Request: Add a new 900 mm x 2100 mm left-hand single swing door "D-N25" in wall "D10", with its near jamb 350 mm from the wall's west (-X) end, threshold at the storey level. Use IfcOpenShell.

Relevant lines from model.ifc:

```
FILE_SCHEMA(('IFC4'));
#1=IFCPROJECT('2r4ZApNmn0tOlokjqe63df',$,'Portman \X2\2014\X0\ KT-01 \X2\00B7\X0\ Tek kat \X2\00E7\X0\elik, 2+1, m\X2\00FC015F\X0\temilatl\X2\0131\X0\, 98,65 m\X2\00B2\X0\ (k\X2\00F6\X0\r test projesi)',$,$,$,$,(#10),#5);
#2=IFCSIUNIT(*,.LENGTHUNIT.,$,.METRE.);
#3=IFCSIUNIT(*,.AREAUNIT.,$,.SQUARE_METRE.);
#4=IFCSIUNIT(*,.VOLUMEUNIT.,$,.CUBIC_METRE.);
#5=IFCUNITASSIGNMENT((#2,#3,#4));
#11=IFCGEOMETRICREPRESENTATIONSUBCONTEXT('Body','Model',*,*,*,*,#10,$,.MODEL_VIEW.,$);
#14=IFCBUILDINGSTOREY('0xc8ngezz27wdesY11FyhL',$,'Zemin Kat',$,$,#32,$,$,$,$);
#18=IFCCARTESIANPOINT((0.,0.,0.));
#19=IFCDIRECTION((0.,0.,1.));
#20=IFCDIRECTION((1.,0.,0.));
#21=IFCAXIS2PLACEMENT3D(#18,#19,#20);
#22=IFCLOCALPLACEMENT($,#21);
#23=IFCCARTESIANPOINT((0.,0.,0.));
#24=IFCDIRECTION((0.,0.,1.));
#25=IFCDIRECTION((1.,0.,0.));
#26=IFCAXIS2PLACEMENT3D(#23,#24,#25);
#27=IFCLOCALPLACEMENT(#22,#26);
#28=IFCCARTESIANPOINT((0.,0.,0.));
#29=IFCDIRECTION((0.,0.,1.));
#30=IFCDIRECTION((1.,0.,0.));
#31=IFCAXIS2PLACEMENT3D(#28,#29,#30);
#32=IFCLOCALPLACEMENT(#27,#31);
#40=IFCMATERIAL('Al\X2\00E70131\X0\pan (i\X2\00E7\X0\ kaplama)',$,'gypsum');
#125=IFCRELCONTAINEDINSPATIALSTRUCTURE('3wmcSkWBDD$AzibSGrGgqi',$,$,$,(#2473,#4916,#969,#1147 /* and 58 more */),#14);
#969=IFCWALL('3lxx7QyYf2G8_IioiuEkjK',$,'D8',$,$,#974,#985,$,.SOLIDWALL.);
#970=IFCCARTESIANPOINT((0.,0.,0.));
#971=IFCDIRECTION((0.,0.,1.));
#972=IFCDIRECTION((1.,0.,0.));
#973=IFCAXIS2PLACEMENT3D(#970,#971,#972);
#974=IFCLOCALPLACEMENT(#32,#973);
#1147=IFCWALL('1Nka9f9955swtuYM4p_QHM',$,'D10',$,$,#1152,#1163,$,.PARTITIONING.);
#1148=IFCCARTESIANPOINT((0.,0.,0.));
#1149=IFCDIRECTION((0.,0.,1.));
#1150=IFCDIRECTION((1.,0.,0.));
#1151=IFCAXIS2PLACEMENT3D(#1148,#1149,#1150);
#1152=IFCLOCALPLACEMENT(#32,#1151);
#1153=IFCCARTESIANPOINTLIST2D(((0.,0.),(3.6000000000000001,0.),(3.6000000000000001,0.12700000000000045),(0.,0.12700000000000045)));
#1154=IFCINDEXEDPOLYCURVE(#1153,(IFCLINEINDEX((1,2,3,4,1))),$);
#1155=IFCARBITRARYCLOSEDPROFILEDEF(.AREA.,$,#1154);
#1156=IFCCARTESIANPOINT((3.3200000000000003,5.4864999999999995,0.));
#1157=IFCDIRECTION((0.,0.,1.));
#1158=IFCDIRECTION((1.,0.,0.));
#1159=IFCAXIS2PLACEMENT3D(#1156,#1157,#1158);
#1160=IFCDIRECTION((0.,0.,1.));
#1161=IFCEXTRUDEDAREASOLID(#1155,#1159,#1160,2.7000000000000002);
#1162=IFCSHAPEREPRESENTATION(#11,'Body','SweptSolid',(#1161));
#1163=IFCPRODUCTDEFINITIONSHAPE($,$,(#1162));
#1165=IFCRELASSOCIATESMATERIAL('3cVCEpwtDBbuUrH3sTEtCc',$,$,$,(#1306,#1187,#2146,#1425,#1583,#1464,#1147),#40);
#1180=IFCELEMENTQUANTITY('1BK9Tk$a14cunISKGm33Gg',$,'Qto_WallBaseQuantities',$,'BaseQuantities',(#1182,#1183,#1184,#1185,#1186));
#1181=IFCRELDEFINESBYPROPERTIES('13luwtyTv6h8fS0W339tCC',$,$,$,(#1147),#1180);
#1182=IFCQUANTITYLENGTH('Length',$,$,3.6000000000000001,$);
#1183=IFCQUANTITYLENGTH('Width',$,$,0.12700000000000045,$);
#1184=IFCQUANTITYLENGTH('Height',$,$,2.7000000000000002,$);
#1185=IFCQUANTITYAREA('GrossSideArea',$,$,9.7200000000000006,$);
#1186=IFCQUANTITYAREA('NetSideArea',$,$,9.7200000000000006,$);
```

```python
import numpy as np
import ifcopenshell
import ifcopenshell.api.feature
import ifcopenshell.api.geometry
import ifcopenshell.api.pset
import ifcopenshell.api.root
import ifcopenshell.api.spatial
import ifcopenshell.geom
import ifcopenshell.util.element
import ifcopenshell.util.placement
import ifcopenshell.util.representation
import ifcopenshell.util.shape
import ifcopenshell.util.unit

model = ifcopenshell.open("model.ifc")
unit_scale = ifcopenshell.util.unit.calculate_unit_scale(model)
area_scale = ifcopenshell.util.unit.calculate_unit_scale(model, "AREAUNIT")
settings = ifcopenshell.geom.settings()


def volume(element):
    """Net volume in cubic metres, openings subtracted."""
    shape = ifcopenshell.geom.create_shape(settings, element)
    return ifcopenshell.util.shape.get_volume(shape.geometry)


wall = model.by_guid("1Nka9f9955swtuYM4p_QHM")
storey = ifcopenshell.util.element.get_container(wall, ifc_class="IfcBuildingStorey")
context = ifcopenshell.util.representation.get_context(model, "Model", "Body", "MODEL_VIEW")
before = volume(wall)

width, height, from_end, sill = 0.9, 2.1, 0.35, 0.0  # metres

# The wall runs along its own X axis, and the end named is its -X end.
wall_shape = ifcopenshell.geom.create_shape(settings, wall)
x, y, z = ifcopenshell.util.shape.get_vertices(wall_shape.geometry).T
start = x.min() + from_end
face, thickness = float(y.min()), float(y.max() - y.min())
wall_matrix = ifcopenshell.util.placement.get_local_placement(wall.ObjectPlacement)
level = ifcopenshell.util.placement.get_local_placement(storey.ObjectPlacement)[2, 3]


def in_wall(x, y):
    """Placement at x, y metres in the wall's axes, at sill height."""
    matrix = wall_matrix.copy()
    matrix[:, 3] = wall_matrix @ np.array([x / unit_scale, y / unit_scale, 0.0, 1.0])
    matrix[2, 3] = level + sill / unit_scale
    return matrix


# Opening: a box that overshoots both wall faces by 50 mm.
opening = ifcopenshell.api.root.create_entity(model, ifc_class="IfcOpeningElement", predefined_type="OPENING")
box = ifcopenshell.api.geometry.add_wall_representation(
    model, context=context, length=width, height=height, thickness=thickness + 0.1
)
ifcopenshell.api.geometry.assign_representation(model, product=opening, representation=box)
ifcopenshell.api.geometry.edit_object_placement(model, product=opening, matrix=in_wall(start, face - 0.05), is_si=False)
ifcopenshell.api.feature.add_feature(model, feature=opening, element=wall)

door = ifcopenshell.api.root.create_entity(model, ifc_class="IfcDoor", name="D-N25", predefined_type="DOOR")
door.OverallWidth, door.OverallHeight = width / unit_scale, height / unit_scale
door.OperationType = "SINGLE_SWING_LEFT"
body = ifcopenshell.api.geometry.add_door_representation(
    model,
    context=context,
    overall_width=door.OverallWidth,
    overall_height=door.OverallHeight,
    operation_type="SINGLE_SWING_LEFT",
    lining_properties={"LiningDepth": thickness / unit_scale, "ThresholdDepth": thickness / unit_scale},
)
ifcopenshell.api.geometry.assign_representation(model, product=door, representation=body)
ifcopenshell.api.spatial.assign_container(model, products=[door], relating_structure=storey)
ifcopenshell.api.feature.add_filling(model, opening=opening, element=door)

# The lining spans the wall, so the door starts at the wall face.
ifcopenshell.api.geometry.edit_object_placement(model, product=door, matrix=in_wall(start, face), is_si=False)

after = volume(wall)

# Update the wall's stored quantities.
qto = model.by_id(ifcopenshell.util.element.get_pset(wall, "Qto_WallBaseQuantities", should_inherit=False)["id"])
ifcopenshell.api.pset.edit_qto(model, qto=qto, properties={"NetSideArea": after / thickness / area_scale})

print(f"wall volume {before:.3f} -> {after:.3f} m3")

model.write("model_v2.ifc")
```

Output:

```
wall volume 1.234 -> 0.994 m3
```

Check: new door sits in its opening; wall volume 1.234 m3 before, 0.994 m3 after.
